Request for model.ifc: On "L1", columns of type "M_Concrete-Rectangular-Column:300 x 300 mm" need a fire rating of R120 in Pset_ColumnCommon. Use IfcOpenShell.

First a look at what the model holds.

```python
import ifcopenshell
import ifcopenshell.util.element

model = ifcopenshell.open("model.ifc")
print(model.schema)
storey = next(s for s in model.by_type("IfcBuildingStorey") if s.Name == "L1")
columns = [e for e in ifcopenshell.util.element.get_decomposition(storey) if e.is_a("IfcColumn")]
seen = {}
for e in columns:
    element_type = ifcopenshell.util.element.get_type(e)
    key = (element_type.Name if element_type != e and element_type else None, ifcopenshell.util.element.get_pset(e, "Pset_ColumnCommon", "FireRating"))
    seen[key] = seen.get(key, 0) + 1
for (name, value), count in sorted(seen.items(), key=str):
    print(count, "x", name, "|", value)
```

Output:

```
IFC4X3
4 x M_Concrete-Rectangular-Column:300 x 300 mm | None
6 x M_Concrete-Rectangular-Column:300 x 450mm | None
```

```python
import ifcopenshell
import ifcopenshell.api.pset
import ifcopenshell.util.element

model = ifcopenshell.open("model.ifc")

storey = next(s for s in model.by_type("IfcBuildingStorey") if s.Name == "L1")
columns = [e for e in ifcopenshell.util.element.get_decomposition(storey) if e.is_a("IfcColumn")]

count = 0
for e in columns:
    element_type = ifcopenshell.util.element.get_type(e)
    if element_type in (None, e) or element_type.Name != "M_Concrete-Rectangular-Column:300 x 300 mm":
        continue
    # add_pset returns the element's existing set when there is one.
    pset = ifcopenshell.api.pset.add_pset(model, product=e, name="Pset_ColumnCommon")
    ifcopenshell.api.pset.edit_pset(model, pset=pset, properties={"FireRating": "R120"})
    count += 1

print(count, "columns updated")

model.write("model_rev.ifc")
```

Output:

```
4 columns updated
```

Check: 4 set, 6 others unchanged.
